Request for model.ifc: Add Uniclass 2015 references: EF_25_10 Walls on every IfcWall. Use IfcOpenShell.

First a look at what the model holds.

```python
import ifcopenshell

model = ifcopenshell.open("model.ifc")
print(model.schema)
print("classifications:", [c.Name for c in model.by_type("IfcClassification")])
for ifc_class in ("IfcDoor", "IfcRoof", "IfcStair", "IfcWall", "IfcWindow"):
    print(ifc_class, len(model.by_type(ifc_class)))
```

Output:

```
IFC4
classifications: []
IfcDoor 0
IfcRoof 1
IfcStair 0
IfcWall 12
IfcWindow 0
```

```python
import ifcopenshell
import ifcopenshell.api.classification

model = ifcopenshell.open("model.ifc")

system = ifcopenshell.api.classification.add_classification(model, classification="Uniclass 2015")

codes = {
    "IfcWall": ("EF_25_10", "Walls"),
}
for ifc_class, (code, name) in codes.items():
    products = model.by_type(ifc_class)
    ifcopenshell.api.classification.add_reference(
        model, products=products, classification=system, identification=code, name=name
    )
    print(code, len(products))

model.write("model_updated.ifc")
```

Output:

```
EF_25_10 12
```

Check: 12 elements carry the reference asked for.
